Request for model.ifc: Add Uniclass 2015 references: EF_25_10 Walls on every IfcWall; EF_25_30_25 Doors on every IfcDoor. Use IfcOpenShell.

First a look at what the model holds.

```python
import ifcopenshell

model = ifcopenshell.open("model.ifc")
print(model.schema)
print("classifications:", [c.Name for c in model.by_type("IfcClassification")])
for ifc_class in ("IfcDoor", "IfcRoof", "IfcStair", "IfcWall", "IfcWindow"):
    print(ifc_class, len(model.by_type(ifc_class)))
```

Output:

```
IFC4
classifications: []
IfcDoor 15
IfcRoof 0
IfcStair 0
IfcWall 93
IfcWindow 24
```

```python
import ifcopenshell
import ifcopenshell.api.classification

model = ifcopenshell.open("model.ifc")

system = ifcopenshell.api.classification.add_classification(model, classification="Uniclass 2015")

codes = {
    "IfcWall": ("EF_25_10", "Walls"),
    "IfcDoor": ("EF_25_30_25", "Doors"),
}
for ifc_class, (code, name) in codes.items():
    products = model.by_type(ifc_class)
    ifcopenshell.api.classification.add_reference(
        model, products=products, classification=system, identification=code, name=name
    )
    print(code, len(products))

model.write("model_edited.ifc")
```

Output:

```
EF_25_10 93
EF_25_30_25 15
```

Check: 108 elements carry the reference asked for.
